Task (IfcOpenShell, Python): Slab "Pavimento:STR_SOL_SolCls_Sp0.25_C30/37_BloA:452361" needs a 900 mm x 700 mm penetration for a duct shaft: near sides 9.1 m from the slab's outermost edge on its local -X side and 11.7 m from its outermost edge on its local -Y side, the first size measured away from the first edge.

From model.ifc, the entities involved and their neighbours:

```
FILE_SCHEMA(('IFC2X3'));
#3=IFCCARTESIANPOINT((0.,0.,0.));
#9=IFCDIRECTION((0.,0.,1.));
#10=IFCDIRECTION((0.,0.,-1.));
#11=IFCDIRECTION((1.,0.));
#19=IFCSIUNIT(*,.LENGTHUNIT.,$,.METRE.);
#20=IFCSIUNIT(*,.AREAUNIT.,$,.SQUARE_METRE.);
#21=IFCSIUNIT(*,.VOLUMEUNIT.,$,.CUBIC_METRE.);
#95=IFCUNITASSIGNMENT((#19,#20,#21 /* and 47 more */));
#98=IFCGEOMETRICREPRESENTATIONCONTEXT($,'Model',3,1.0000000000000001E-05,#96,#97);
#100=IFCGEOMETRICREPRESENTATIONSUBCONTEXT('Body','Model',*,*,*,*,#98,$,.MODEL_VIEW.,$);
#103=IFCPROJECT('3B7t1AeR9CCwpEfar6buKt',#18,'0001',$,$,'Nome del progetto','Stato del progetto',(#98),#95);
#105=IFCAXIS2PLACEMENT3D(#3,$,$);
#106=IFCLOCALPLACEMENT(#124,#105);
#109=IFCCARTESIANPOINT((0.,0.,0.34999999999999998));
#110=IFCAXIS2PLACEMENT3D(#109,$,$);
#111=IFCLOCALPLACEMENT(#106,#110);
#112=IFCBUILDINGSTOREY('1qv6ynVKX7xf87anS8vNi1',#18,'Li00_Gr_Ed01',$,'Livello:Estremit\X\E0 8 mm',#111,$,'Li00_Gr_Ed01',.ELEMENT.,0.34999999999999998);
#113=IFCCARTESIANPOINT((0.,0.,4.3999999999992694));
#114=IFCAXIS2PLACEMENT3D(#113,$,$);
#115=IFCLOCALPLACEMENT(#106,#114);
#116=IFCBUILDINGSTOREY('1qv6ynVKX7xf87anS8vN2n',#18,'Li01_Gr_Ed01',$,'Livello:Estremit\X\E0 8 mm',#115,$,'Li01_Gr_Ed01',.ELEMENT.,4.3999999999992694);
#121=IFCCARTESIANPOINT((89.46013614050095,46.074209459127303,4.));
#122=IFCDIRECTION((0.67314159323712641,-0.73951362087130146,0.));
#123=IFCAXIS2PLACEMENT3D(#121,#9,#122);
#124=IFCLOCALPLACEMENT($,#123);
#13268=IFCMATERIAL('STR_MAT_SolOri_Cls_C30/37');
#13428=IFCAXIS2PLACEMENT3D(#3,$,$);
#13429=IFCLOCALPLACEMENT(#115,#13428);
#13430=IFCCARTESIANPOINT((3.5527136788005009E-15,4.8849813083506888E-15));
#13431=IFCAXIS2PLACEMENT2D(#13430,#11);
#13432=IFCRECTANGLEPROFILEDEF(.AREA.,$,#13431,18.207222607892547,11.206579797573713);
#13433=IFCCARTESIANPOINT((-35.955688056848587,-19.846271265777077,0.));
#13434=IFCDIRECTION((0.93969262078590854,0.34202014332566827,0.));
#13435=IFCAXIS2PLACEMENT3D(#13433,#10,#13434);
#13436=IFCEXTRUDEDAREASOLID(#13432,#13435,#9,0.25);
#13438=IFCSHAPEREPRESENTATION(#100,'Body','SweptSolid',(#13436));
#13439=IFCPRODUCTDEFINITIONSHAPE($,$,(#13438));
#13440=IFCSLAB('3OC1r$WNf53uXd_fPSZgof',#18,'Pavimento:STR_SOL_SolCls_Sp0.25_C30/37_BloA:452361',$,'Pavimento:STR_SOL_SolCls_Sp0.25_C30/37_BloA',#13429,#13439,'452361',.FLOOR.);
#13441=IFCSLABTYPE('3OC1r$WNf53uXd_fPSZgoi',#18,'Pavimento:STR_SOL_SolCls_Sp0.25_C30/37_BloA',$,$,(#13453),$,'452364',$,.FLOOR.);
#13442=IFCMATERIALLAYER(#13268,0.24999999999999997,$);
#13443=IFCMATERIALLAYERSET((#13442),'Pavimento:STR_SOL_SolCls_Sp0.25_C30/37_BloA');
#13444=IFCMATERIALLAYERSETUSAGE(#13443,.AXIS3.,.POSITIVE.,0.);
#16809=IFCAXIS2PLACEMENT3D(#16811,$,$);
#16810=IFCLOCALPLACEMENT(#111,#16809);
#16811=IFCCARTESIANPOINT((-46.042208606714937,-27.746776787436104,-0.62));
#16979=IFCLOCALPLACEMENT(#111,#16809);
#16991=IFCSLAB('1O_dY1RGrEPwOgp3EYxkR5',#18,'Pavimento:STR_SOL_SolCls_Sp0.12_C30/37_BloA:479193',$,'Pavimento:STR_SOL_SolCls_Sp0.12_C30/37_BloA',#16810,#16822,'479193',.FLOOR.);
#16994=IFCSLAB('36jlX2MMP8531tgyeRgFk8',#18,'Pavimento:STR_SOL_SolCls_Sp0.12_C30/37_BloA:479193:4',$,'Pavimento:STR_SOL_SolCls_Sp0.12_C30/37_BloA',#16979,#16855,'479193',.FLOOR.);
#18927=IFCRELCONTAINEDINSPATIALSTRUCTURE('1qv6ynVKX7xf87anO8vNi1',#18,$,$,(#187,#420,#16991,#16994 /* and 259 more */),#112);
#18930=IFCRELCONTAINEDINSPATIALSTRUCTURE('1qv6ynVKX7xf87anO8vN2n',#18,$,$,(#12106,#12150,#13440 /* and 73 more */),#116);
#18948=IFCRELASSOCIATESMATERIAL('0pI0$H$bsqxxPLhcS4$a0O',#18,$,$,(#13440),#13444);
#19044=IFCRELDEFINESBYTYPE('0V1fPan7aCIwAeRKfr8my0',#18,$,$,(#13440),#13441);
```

```python
import numpy as np
import ifcopenshell
import ifcopenshell.api.feature
import ifcopenshell.api.geometry
import ifcopenshell.api.root
import ifcopenshell.geom
import ifcopenshell.util.placement
import ifcopenshell.util.representation
import ifcopenshell.util.shape
import ifcopenshell.util.unit

model = ifcopenshell.open("model.ifc")
unit_scale = ifcopenshell.util.unit.calculate_unit_scale(model)
settings = ifcopenshell.geom.settings()


def volume(element):
    """Net volume in cubic metres, openings subtracted."""
    shape = ifcopenshell.geom.create_shape(settings, element)
    return ifcopenshell.util.shape.get_volume(shape.geometry)


slab = model.by_guid("3OC1r$WNf53uXd_fPSZgof")
before = volume(slab)

# Extent in the slab's own axes, in metres. The edges named are its -X and -Y sides.
slab_shape = ifcopenshell.geom.create_shape(settings, slab)
vertices = ifcopenshell.util.shape.get_vertices(slab_shape.geometry)
x_min, y_min, bottom = vertices.min(axis=0)
top = vertices[:, 2].max()

opening = ifcopenshell.api.root.create_entity(model, ifc_class="IfcOpeningElement", name="Duct shaft opening")
context = ifcopenshell.util.representation.get_context(model, "Model", "Body", "MODEL_VIEW")
width, depth = 0.9, 0.7
outline = [(0.0, 0.0), (width, 0.0), (width, depth), (0.0, depth), (0.0, 0.0)]
# Overshoot both faces by 50 mm so the cut is clean.
shape = ifcopenshell.api.geometry.add_slab_representation(
    model, context=context, depth=top - bottom + 0.1, polyline=outline
)
ifcopenshell.api.geometry.assign_representation(model, product=opening, representation=shape)

matrix = ifcopenshell.util.placement.get_local_placement(slab.ObjectPlacement)
matrix[:, 3] = matrix @ np.append(np.array([x_min + 9.1, y_min + 11.7, bottom - 0.05]) / unit_scale, 1.0)
ifcopenshell.api.geometry.edit_object_placement(model, product=opening, matrix=matrix, is_si=False)
ifcopenshell.api.feature.add_feature(model, feature=opening, element=slab)

after = volume(slab)

print(f"slab volume {before:.3f} -> {after:.3f} m3")

model.write("model_rev.ifc")
```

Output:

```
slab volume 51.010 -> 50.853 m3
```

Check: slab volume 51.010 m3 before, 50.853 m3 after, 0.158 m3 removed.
